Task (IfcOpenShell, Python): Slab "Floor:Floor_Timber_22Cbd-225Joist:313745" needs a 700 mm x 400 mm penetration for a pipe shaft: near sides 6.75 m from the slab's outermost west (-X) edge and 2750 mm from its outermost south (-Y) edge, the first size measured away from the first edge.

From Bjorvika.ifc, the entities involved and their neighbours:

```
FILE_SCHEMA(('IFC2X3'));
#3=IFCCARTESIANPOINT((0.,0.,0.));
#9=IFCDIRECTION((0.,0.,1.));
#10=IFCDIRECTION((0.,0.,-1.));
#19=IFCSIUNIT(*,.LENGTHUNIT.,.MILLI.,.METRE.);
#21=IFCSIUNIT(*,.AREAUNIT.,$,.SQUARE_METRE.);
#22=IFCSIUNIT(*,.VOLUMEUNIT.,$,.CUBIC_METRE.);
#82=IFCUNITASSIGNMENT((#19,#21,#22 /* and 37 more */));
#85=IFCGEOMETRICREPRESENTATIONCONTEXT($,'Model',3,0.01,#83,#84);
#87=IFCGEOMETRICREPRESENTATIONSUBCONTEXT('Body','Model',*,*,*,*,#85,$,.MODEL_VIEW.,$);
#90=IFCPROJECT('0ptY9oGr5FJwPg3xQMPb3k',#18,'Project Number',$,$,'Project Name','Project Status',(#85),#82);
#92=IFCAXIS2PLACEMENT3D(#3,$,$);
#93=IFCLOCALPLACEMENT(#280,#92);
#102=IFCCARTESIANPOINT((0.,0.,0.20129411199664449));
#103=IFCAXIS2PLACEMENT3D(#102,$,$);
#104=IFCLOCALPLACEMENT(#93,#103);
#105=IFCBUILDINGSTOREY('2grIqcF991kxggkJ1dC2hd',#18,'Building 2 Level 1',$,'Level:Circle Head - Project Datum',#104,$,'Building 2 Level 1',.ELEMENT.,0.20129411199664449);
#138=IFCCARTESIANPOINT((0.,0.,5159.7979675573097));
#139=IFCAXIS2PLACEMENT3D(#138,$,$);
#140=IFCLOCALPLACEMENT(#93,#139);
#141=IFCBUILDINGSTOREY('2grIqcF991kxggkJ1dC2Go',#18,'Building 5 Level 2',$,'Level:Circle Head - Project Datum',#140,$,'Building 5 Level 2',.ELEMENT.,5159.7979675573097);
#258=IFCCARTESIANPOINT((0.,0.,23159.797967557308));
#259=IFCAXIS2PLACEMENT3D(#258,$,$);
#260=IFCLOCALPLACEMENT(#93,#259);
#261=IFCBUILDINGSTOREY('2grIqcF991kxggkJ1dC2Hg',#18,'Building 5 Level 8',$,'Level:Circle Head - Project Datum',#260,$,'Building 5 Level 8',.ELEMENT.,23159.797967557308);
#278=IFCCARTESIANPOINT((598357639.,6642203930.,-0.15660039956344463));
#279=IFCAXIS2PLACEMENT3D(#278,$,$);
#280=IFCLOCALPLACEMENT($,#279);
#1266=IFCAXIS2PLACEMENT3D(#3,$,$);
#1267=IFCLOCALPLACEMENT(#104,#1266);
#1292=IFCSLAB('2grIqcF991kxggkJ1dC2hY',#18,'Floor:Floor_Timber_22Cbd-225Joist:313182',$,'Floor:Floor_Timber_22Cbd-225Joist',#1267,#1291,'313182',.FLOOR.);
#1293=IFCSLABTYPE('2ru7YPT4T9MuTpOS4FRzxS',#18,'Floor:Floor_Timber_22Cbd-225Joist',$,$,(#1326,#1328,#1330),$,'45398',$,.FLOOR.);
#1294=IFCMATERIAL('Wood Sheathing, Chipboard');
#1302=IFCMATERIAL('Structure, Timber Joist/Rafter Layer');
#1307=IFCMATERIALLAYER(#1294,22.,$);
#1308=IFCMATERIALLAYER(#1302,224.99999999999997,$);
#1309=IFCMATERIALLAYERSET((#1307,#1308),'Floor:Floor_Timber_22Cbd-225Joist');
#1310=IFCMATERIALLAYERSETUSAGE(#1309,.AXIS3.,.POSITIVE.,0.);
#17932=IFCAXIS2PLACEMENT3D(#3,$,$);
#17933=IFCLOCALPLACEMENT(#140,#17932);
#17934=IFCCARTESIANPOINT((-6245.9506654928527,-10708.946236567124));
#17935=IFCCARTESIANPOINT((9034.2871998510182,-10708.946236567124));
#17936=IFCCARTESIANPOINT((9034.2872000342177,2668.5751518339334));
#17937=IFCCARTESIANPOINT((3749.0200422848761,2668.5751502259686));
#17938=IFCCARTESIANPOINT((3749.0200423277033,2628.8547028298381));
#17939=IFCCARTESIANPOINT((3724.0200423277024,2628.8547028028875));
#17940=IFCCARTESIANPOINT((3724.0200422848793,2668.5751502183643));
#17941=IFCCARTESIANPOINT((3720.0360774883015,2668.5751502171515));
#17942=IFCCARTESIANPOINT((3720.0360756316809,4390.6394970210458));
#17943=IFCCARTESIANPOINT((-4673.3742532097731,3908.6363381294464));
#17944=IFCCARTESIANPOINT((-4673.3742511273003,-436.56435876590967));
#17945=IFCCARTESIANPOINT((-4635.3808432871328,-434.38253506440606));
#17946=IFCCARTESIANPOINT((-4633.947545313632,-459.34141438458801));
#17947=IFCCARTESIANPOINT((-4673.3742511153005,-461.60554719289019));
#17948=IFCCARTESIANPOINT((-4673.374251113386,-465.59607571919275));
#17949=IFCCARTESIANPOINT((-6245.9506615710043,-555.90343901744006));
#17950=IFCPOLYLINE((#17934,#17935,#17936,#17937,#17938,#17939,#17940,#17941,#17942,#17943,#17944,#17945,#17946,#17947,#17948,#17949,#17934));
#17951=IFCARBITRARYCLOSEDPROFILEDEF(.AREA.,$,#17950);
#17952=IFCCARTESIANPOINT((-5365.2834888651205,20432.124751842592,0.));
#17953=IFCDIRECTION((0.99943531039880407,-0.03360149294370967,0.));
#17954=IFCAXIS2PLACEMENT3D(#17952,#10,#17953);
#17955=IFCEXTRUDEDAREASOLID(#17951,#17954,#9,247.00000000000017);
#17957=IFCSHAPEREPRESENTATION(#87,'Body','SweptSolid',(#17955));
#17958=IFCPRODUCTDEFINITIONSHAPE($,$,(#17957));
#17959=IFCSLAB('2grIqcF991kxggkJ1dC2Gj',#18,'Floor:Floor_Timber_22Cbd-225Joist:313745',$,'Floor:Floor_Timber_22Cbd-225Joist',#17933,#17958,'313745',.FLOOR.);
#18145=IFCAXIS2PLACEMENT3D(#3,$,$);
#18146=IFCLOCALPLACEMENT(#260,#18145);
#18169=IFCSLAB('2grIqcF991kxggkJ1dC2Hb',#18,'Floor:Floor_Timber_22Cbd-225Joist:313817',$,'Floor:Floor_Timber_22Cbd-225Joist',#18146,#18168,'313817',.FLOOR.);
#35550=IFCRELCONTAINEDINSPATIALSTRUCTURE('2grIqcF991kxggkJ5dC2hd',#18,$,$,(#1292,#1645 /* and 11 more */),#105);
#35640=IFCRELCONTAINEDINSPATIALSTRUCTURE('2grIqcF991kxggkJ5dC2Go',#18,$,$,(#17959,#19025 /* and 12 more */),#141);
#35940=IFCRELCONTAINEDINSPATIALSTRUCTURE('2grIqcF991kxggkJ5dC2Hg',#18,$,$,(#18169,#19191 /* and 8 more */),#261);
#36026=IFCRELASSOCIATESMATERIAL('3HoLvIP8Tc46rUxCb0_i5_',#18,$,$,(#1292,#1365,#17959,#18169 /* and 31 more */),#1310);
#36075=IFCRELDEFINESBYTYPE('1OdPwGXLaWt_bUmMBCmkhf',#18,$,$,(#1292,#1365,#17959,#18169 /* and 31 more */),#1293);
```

```python
import numpy as np
import ifcopenshell
import ifcopenshell.api.feature
import ifcopenshell.api.geometry
import ifcopenshell.api.root
import ifcopenshell.geom
import ifcopenshell.util.placement
import ifcopenshell.util.representation
import ifcopenshell.util.shape
import ifcopenshell.util.unit

model = ifcopenshell.open("Bjorvika.ifc")
unit_scale = ifcopenshell.util.unit.calculate_unit_scale(model)
settings = ifcopenshell.geom.settings()


def volume(element):
    """Net volume in cubic metres, openings subtracted."""
    shape = ifcopenshell.geom.create_shape(settings, element)
    return ifcopenshell.util.shape.get_volume(shape.geometry)


slab = model.by_guid("2grIqcF991kxggkJ1dC2Gj")
before = volume(slab)

# Extent in the slab's own axes, in metres. The edges named are its -X and -Y sides.
slab_shape = ifcopenshell.geom.create_shape(settings, slab)
vertices = ifcopenshell.util.shape.get_vertices(slab_shape.geometry)
x_min, y_min, bottom = vertices.min(axis=0)
top = vertices[:, 2].max()

opening = ifcopenshell.api.root.create_entity(model, ifc_class="IfcOpeningElement", name="Pipe shaft opening")
context = ifcopenshell.util.representation.get_context(model, "Model", "Body", "MODEL_VIEW")
width, depth = 0.7, 0.4
outline = [(0.0, 0.0), (width, 0.0), (width, depth), (0.0, depth), (0.0, 0.0)]
# Overshoot both faces by 50 mm so the cut is clean.
shape = ifcopenshell.api.geometry.add_slab_representation(
    model, context=context, depth=top - bottom + 0.1, polyline=outline
)
ifcopenshell.api.geometry.assign_representation(model, product=opening, representation=shape)

matrix = ifcopenshell.util.placement.get_local_placement(slab.ObjectPlacement)
matrix[:, 3] = matrix @ np.append(np.array([x_min + 6.75, y_min + 2.75, bottom - 0.05]) / unit_scale, 1.0)
ifcopenshell.api.geometry.edit_object_placement(model, product=opening, matrix=matrix, is_si=False)
ifcopenshell.api.feature.add_feature(model, feature=opening, element=slab)

after = volume(slab)

print(f"slab volume {before:.3f} -> {after:.3f} m3")

model.write("Bjorvika-out.ifc")
```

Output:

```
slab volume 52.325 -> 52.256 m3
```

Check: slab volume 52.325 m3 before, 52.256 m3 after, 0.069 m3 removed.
